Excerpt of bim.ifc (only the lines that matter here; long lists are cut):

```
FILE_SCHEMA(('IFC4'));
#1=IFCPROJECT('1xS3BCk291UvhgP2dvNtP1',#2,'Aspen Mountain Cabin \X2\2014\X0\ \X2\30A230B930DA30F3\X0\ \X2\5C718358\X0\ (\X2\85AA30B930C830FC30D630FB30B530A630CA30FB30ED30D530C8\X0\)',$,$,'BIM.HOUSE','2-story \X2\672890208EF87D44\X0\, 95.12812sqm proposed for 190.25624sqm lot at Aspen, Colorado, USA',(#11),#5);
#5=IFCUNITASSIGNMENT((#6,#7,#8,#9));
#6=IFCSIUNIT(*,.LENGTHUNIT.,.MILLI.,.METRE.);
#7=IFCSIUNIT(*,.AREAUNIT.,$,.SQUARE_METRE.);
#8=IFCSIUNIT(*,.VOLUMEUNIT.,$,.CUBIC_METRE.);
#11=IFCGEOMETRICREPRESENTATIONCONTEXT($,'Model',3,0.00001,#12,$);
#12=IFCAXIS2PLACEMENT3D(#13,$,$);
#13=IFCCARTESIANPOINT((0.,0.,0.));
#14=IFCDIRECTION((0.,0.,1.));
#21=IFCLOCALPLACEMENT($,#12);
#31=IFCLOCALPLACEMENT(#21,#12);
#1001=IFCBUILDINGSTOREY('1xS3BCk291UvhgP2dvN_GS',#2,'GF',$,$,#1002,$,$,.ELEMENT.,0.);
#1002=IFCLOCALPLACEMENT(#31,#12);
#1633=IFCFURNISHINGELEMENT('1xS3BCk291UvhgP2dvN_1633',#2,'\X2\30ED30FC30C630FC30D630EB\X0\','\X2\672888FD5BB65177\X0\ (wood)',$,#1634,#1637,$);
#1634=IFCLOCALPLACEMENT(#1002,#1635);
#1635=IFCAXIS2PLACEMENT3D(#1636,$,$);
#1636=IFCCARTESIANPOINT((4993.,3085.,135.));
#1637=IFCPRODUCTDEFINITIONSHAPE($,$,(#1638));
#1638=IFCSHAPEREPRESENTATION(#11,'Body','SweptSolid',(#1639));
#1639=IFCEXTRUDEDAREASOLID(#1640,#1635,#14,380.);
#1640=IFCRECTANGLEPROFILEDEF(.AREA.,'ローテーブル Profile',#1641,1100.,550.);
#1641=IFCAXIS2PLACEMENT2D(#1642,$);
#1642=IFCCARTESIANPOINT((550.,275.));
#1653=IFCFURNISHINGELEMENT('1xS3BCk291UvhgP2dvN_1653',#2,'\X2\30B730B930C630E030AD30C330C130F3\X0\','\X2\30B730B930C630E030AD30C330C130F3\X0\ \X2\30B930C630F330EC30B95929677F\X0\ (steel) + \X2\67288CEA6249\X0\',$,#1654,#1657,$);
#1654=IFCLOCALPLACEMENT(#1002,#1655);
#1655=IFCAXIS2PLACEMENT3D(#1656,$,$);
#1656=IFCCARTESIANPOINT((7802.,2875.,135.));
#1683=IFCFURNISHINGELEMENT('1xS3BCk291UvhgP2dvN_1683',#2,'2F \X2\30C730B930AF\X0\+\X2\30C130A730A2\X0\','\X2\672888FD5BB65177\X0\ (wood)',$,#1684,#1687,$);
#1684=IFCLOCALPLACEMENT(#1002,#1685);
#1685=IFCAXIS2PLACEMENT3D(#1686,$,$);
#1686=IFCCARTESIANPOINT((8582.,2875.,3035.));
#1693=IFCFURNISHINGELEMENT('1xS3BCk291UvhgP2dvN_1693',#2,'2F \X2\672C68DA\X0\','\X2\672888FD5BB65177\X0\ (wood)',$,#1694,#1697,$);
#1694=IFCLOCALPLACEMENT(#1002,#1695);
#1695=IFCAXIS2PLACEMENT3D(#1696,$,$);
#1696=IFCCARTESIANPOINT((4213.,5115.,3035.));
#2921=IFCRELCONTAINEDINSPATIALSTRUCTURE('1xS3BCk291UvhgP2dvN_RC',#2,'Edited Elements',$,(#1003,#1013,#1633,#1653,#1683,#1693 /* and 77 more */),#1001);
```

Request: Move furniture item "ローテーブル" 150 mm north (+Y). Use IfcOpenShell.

```python
import ifcopenshell
import ifcopenshell.api.geometry
import ifcopenshell.util.placement
import ifcopenshell.util.unit

model = ifcopenshell.open("bim.ifc")
unit_scale = ifcopenshell.util.unit.calculate_unit_scale(model)

item = model.by_guid("1xS3BCk291UvhgP2dvN_1633")
matrix = ifcopenshell.util.placement.get_local_placement(item.ObjectPlacement)
matrix[1, 3] += 0.15 / unit_scale
ifcopenshell.api.geometry.edit_object_placement(model, product=item, matrix=matrix, is_si=False)

print(ifcopenshell.util.placement.get_local_placement(item.ObjectPlacement).round(3) + 0.0)

model.write("bim_updated.ifc")
```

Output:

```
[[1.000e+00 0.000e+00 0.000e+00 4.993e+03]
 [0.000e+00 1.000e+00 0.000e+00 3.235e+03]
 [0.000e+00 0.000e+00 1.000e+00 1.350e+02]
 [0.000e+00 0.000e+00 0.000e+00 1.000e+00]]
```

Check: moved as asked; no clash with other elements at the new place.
